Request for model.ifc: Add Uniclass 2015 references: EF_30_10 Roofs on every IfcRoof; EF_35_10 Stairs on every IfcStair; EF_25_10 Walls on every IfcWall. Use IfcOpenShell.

First a look at what the model holds.

```python
import ifcopenshell

model = ifcopenshell.open("model.ifc")
print(model.schema)
print("classifications:", [c.Name for c in model.by_type("IfcClassification")])
for ifc_class in ("IfcDoor", "IfcRoof", "IfcStair", "IfcWall", "IfcWindow"):
    print(ifc_class, len(model.by_type(ifc_class)))
```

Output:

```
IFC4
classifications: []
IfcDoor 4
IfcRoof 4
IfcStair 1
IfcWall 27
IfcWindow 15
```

```python
import ifcopenshell
import ifcopenshell.api.classification

model = ifcopenshell.open("model.ifc")

system = ifcopenshell.api.classification.add_classification(model, classification="Uniclass 2015")

codes = {
    "IfcRoof": ("EF_30_10", "Roofs"),
    "IfcStair": ("EF_35_10", "Stairs"),
    "IfcWall": ("EF_25_10", "Walls"),
}
for ifc_class, (code, name) in codes.items():
    products = model.by_type(ifc_class)
    ifcopenshell.api.classification.add_reference(
        model, products=products, classification=system, identification=code, name=name
    )
    print(code, len(products))

model.write("model_v2.ifc")
```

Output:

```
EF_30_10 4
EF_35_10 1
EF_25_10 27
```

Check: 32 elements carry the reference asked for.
